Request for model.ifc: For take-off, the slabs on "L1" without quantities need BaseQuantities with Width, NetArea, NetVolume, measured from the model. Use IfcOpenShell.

First a look at what the model holds.

```python
import ifcopenshell
import ifcopenshell.util.element
import ifcopenshell.util.unit

model = ifcopenshell.open("model.ifc")
print(model.schema)
for unit_type in ("LENGTHUNIT", "AREAUNIT", "VOLUMEUNIT"):
    print(unit_type, ifcopenshell.util.unit.calculate_unit_scale(model, unit_type))
storey = next(s for s in model.by_type("IfcBuildingStorey") if s.Name == "L1")
slabs = [e for e in ifcopenshell.util.element.get_decomposition(storey) if e.is_a("IfcSlab")]
for e in sorted(slabs, key=lambda e: e.id()):
    print(e.id(), e.is_a(), e.Name, list(ifcopenshell.util.element.get_psets(e, qtos_only=True)), sep=" | ")
```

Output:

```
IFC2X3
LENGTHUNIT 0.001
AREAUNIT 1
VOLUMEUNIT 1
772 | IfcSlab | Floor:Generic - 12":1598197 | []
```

```python
import ifcopenshell
import ifcopenshell.api.pset
import ifcopenshell.geom
import ifcopenshell.util.element
import ifcopenshell.util.shape
import ifcopenshell.util.unit

model = ifcopenshell.open("model.ifc")
unit_scale = ifcopenshell.util.unit.calculate_unit_scale(model)
area_scale = ifcopenshell.util.unit.calculate_unit_scale(model, "AREAUNIT")
volume_scale = ifcopenshell.util.unit.calculate_unit_scale(model, "VOLUMEUNIT")
settings = ifcopenshell.geom.settings()

storey = next(s for s in model.by_type("IfcBuildingStorey") if s.Name == "L1")
slabs = [e for e in ifcopenshell.util.element.get_decomposition(storey) if e.is_a("IfcSlab")]

for e in sorted(slabs, key=lambda e: e.id()):
    if ifcopenshell.util.element.get_psets(e, qtos_only=True, should_inherit=False):
        continue
    # Geometry comes back in metres, in the element's own axes.
    shape = ifcopenshell.geom.create_shape(settings, e)
    values = {
        "Width": ifcopenshell.util.shape.get_z(shape.geometry) / unit_scale,
        "NetArea": ifcopenshell.util.shape.get_footprint_area(shape.geometry) / area_scale,
        "NetVolume": ifcopenshell.util.shape.get_volume(shape.geometry) / volume_scale,
    }
    qto = ifcopenshell.api.pset.add_qto(model, product=e, name="BaseQuantities")
    ifcopenshell.api.pset.edit_qto(model, qto=qto, properties=values)
    print(e.id(), {k: round(v, 3) for k, v in values.items()})

model.write("model_v2.ifc")
```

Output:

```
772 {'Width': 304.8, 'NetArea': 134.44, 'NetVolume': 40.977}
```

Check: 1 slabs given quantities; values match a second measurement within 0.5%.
